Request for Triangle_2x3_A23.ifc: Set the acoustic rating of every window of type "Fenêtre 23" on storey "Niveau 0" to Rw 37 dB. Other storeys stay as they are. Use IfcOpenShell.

First a look at what the model holds.

```python
import ifcopenshell
import ifcopenshell.util.element

model = ifcopenshell.open("Triangle_2x3_A23.ifc")
print(model.schema)
storey = next(s for s in model.by_type("IfcBuildingStorey") if s.Name == "Niveau 0")
windows = [e for e in ifcopenshell.util.element.get_decomposition(storey) if e.is_a("IfcWindow")]
seen = {}
for e in windows:
    element_type = ifcopenshell.util.element.get_type(e)
    key = (element_type.Name if element_type != e and element_type else None, ifcopenshell.util.element.get_pset(e, "Pset_WindowCommon", "AcousticRating"))
    seen[key] = seen.get(key, 0) + 1
for (name, value), count in sorted(seen.items(), key=str):
    print(count, "x", name, "|", value)
```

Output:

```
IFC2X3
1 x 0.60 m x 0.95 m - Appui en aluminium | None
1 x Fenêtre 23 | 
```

```python
import ifcopenshell
import ifcopenshell.api.pset
import ifcopenshell.util.element

model = ifcopenshell.open("Triangle_2x3_A23.ifc")

storey = next(s for s in model.by_type("IfcBuildingStorey") if s.Name == "Niveau 0")
windows = [e for e in ifcopenshell.util.element.get_decomposition(storey) if e.is_a("IfcWindow")]

count = 0
for e in windows:
    element_type = ifcopenshell.util.element.get_type(e)
    if element_type in (None, e) or element_type.Name != "Fenêtre 23":
        continue
    # add_pset returns the element's existing set when there is one.
    pset = ifcopenshell.api.pset.add_pset(model, product=e, name="Pset_WindowCommon")
    ifcopenshell.api.pset.edit_pset(model, pset=pset, properties={"AcousticRating": "Rw 37 dB"})
    count += 1

print(count, "windows updated")

model.write("Triangle_2x3_A23_edited.ifc")
```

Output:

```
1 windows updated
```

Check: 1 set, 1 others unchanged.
